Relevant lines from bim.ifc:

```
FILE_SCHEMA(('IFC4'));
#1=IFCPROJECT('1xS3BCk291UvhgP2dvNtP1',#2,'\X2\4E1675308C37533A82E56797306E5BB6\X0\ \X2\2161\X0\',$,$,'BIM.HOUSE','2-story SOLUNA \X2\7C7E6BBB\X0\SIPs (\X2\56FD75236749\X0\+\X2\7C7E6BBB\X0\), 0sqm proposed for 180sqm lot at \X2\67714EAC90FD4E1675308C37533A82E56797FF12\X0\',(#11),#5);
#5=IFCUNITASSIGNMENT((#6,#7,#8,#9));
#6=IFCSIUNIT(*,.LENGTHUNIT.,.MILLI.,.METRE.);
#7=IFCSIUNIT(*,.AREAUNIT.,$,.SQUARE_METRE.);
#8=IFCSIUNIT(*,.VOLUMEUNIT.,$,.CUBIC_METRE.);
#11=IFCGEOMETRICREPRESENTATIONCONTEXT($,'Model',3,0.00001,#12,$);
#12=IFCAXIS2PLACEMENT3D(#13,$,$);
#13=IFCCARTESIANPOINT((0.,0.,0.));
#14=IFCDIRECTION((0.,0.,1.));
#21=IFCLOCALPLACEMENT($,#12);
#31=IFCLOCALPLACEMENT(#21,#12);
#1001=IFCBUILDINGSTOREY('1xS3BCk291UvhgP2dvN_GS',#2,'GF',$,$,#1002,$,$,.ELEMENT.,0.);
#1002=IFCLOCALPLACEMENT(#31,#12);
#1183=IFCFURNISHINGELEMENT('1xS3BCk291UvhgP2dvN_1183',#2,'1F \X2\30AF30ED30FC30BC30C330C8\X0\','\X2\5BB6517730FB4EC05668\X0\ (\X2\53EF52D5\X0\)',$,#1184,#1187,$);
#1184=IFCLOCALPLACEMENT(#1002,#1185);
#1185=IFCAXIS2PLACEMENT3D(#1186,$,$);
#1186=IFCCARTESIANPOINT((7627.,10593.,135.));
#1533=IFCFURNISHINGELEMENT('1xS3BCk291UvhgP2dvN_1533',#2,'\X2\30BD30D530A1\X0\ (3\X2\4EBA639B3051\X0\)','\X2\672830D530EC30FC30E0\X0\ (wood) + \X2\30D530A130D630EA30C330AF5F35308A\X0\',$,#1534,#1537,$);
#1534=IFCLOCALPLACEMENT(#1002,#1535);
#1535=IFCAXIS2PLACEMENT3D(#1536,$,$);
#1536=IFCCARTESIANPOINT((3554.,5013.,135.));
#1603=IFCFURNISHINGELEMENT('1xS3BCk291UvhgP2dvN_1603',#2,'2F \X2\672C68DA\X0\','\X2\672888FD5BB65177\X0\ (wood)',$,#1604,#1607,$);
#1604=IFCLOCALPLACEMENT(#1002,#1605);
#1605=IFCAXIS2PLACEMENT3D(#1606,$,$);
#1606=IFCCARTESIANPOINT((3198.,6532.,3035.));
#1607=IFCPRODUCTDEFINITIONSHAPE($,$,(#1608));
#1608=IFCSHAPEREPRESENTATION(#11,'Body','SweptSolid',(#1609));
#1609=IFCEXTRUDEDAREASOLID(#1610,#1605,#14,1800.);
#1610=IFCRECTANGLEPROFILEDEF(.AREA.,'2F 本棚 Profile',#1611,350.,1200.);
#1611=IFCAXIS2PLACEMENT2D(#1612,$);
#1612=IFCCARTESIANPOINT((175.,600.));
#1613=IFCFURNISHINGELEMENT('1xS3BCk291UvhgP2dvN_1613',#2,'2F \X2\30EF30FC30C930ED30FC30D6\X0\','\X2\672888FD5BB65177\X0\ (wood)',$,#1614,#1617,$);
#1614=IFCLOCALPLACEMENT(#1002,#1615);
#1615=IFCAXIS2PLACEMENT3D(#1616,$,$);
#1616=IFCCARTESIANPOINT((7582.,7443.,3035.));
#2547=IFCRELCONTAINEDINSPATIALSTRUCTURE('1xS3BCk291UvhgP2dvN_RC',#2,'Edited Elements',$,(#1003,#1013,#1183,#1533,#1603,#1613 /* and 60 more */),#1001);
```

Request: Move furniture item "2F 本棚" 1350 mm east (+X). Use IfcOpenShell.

```python
import ifcopenshell
import ifcopenshell.api.geometry
import ifcopenshell.util.placement
import ifcopenshell.util.unit

model = ifcopenshell.open("bim.ifc")
unit_scale = ifcopenshell.util.unit.calculate_unit_scale(model)

item = model.by_id(1603)
matrix = ifcopenshell.util.placement.get_local_placement(item.ObjectPlacement)
matrix[0, 3] += 1.35 / unit_scale
ifcopenshell.api.geometry.edit_object_placement(model, product=item, matrix=matrix, is_si=False)

print(ifcopenshell.util.placement.get_local_placement(item.ObjectPlacement).round(3) + 0.0)

model.write("bim_edited.ifc")
```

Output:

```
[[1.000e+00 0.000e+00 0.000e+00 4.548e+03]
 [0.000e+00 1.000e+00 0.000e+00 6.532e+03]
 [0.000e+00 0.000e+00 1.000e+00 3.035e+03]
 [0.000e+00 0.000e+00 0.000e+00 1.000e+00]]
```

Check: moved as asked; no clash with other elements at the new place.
